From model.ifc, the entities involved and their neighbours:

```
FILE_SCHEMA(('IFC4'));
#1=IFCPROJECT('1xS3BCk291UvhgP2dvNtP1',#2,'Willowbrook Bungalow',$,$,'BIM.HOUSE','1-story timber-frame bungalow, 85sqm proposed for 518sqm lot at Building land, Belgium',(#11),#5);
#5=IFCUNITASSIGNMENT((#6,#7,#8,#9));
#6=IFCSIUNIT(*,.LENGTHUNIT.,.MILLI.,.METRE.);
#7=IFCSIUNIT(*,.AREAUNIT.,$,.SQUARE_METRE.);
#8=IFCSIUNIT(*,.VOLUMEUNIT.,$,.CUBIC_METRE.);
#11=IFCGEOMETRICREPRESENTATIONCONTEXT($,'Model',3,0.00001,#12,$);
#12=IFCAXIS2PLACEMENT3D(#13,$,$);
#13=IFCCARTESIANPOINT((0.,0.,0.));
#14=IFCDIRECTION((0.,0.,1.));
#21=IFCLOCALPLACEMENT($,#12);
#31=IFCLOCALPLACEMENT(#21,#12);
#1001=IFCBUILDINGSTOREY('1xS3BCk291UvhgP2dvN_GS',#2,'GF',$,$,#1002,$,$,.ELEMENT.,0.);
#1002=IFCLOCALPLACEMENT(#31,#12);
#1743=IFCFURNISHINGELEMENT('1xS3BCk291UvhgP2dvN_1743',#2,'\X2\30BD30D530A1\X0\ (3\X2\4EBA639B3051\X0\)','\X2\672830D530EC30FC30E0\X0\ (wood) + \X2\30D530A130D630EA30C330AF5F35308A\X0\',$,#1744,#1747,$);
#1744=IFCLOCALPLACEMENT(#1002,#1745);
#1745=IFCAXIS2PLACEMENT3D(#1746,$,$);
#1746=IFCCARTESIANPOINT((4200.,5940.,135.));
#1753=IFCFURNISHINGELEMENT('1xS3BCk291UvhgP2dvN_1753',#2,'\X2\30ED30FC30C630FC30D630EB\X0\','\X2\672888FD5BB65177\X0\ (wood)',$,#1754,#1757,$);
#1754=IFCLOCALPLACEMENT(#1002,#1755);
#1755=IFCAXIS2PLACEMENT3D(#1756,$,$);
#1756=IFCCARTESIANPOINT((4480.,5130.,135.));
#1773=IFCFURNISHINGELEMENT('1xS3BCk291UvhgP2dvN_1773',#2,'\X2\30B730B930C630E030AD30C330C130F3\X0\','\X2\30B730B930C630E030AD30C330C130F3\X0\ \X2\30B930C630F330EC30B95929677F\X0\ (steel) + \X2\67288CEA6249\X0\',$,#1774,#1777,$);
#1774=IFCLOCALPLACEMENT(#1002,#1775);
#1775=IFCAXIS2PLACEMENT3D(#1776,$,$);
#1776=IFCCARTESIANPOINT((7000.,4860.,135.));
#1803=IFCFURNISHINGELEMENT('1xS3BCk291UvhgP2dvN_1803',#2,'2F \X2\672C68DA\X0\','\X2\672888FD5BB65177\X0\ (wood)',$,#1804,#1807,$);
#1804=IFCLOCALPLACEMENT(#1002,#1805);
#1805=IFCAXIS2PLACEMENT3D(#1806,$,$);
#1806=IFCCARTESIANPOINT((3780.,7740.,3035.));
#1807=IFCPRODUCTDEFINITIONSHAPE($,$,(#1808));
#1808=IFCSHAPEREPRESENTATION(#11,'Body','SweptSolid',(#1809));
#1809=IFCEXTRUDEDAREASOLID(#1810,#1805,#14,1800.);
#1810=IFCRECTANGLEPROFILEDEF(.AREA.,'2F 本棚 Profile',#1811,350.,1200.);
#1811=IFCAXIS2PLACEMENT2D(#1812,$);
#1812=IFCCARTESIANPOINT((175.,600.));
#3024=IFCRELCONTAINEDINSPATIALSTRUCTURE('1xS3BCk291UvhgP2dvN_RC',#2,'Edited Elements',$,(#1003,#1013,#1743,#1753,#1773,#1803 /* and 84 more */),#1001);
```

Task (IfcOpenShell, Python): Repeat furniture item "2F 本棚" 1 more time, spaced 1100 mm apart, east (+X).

```python
import numpy as np
import ifcopenshell
import ifcopenshell.api.geometry
import ifcopenshell.api.root
import ifcopenshell.util.element
import ifcopenshell.util.placement
import ifcopenshell.util.unit

model = ifcopenshell.open("model.ifc")
unit_scale = ifcopenshell.util.unit.calculate_unit_scale(model)


def reuse_history(source, copy):
    """copy_class also copies each property set's owner history, people and application; keep the originals."""
    for rel in copy.IsDefinedBy:
        if rel.is_a("IfcRelDefinesByProperties") and (history := rel.RelatingPropertyDefinition.OwnerHistory):
            rel.RelatingPropertyDefinition.OwnerHistory = source.OwnerHistory
            ifcopenshell.util.element.remove_deep2(model, history)


source = model.by_id(1803)
base = ifcopenshell.util.placement.get_local_placement(source.ObjectPlacement)
step = np.array([1.0, 0.0, 0.0]) * 1.1 / unit_scale

for i in range(1, 2):
    copy = ifcopenshell.api.root.copy_class(model, product=source)
    copy.Representation = ifcopenshell.util.element.copy_deep(
        model, source.Representation, exclude=["IfcGeometricRepresentationContext", "IfcRepresentationMap"]
    )
    reuse_history(source, copy)
    matrix = base.copy()
    matrix[:3, 3] += i * step
    print("added at", matrix[:3, 3].round(3) + 0.0)
    ifcopenshell.api.geometry.edit_object_placement(model, product=copy, matrix=matrix, is_si=False)

model.write("model-out.ifc")
```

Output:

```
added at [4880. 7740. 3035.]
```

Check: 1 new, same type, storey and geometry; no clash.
